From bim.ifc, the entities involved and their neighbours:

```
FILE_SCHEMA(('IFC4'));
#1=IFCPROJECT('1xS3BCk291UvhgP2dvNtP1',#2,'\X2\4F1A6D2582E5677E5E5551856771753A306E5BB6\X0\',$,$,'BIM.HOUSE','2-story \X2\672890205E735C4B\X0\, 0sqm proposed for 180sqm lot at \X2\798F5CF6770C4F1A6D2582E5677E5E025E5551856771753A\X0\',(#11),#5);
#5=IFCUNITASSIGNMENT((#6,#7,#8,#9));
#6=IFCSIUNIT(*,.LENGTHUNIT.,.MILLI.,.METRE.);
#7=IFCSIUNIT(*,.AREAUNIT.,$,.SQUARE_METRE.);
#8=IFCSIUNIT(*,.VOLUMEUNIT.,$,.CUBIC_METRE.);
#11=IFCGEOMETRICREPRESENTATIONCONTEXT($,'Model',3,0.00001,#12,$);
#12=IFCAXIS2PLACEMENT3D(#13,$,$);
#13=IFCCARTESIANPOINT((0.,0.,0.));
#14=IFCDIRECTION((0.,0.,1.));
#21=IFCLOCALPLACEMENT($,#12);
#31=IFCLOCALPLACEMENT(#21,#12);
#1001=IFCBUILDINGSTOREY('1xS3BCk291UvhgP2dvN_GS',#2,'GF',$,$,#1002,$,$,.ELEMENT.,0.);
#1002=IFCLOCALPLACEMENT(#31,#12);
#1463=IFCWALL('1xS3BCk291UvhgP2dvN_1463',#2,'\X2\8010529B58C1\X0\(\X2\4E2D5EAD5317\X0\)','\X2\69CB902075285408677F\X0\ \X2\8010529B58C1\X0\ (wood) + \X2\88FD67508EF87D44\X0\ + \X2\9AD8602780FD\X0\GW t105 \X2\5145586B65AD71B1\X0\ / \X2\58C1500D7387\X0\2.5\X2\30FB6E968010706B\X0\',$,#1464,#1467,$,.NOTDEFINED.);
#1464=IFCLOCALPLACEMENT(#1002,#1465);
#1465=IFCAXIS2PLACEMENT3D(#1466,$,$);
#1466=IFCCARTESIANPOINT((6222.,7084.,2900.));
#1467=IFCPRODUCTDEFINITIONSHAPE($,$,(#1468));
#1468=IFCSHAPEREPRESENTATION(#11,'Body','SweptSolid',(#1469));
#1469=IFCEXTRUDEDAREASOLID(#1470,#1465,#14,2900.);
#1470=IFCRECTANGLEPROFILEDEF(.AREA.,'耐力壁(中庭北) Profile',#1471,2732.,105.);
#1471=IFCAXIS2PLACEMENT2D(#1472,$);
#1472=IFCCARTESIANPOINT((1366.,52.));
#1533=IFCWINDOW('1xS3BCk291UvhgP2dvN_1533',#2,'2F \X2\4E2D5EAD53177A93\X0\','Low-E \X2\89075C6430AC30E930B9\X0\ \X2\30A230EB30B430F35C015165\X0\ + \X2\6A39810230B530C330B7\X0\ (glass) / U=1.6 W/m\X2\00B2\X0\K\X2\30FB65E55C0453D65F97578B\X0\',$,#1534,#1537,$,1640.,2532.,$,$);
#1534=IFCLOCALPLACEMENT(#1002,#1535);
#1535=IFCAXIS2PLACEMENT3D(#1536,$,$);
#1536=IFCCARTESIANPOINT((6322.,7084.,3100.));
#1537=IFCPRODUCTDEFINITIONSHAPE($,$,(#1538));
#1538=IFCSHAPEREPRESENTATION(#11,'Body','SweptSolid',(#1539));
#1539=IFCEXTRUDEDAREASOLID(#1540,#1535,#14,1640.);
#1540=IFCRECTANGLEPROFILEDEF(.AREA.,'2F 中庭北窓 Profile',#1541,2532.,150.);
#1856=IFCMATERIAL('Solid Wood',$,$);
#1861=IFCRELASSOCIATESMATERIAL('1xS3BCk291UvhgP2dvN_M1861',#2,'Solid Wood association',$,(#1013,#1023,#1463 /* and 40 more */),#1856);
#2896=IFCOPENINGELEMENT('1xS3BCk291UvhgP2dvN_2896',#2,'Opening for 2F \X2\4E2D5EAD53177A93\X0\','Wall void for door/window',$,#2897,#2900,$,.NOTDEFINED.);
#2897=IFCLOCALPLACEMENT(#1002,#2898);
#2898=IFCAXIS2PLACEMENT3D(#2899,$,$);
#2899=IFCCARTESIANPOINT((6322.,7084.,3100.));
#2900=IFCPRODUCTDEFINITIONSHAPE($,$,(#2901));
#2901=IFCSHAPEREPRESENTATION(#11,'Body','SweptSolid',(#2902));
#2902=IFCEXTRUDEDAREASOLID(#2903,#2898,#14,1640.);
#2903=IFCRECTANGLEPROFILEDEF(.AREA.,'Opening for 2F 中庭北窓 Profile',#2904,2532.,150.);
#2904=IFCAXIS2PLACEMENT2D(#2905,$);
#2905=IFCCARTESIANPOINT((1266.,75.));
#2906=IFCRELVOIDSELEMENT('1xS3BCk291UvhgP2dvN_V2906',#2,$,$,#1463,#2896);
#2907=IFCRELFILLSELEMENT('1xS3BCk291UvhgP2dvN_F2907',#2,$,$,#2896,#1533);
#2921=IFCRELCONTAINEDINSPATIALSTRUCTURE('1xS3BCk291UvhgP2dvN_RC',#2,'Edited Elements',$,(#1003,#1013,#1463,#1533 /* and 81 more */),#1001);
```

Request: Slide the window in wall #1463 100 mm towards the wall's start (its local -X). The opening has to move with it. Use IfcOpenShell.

```python
import ifcopenshell
import ifcopenshell.api.geometry
import ifcopenshell.util.placement
import ifcopenshell.util.unit

model = ifcopenshell.open("bim.ifc")
unit_scale = ifcopenshell.util.unit.calculate_unit_scale(model)

window = model.by_id(1533)
opening = window.FillsVoids[0].RelatingOpeningElement
wall = opening.VoidsElements[0].RelatingBuildingElement

wall_matrix = ifcopenshell.util.placement.get_local_placement(wall.ObjectPlacement)
shift = wall_matrix[:3, 0] * -0.1 / unit_scale
before = ifcopenshell.util.placement.get_local_placement(window.ObjectPlacement)[:3, 3].copy()

# The window is not placed relative to its opening, so move both.
for product in (opening, window):
    matrix = ifcopenshell.util.placement.get_local_placement(product.ObjectPlacement)
    matrix[:3, 3] += shift
    ifcopenshell.api.geometry.edit_object_placement(model, product=product, matrix=matrix, is_si=False)

after = ifcopenshell.util.placement.get_local_placement(window.ObjectPlacement)[:3, 3]
print("window moved by", (after - before).round(3) + 0.0)

model.write("bim-out.ifc")
```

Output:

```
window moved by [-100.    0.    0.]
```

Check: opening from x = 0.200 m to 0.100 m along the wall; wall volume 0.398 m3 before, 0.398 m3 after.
